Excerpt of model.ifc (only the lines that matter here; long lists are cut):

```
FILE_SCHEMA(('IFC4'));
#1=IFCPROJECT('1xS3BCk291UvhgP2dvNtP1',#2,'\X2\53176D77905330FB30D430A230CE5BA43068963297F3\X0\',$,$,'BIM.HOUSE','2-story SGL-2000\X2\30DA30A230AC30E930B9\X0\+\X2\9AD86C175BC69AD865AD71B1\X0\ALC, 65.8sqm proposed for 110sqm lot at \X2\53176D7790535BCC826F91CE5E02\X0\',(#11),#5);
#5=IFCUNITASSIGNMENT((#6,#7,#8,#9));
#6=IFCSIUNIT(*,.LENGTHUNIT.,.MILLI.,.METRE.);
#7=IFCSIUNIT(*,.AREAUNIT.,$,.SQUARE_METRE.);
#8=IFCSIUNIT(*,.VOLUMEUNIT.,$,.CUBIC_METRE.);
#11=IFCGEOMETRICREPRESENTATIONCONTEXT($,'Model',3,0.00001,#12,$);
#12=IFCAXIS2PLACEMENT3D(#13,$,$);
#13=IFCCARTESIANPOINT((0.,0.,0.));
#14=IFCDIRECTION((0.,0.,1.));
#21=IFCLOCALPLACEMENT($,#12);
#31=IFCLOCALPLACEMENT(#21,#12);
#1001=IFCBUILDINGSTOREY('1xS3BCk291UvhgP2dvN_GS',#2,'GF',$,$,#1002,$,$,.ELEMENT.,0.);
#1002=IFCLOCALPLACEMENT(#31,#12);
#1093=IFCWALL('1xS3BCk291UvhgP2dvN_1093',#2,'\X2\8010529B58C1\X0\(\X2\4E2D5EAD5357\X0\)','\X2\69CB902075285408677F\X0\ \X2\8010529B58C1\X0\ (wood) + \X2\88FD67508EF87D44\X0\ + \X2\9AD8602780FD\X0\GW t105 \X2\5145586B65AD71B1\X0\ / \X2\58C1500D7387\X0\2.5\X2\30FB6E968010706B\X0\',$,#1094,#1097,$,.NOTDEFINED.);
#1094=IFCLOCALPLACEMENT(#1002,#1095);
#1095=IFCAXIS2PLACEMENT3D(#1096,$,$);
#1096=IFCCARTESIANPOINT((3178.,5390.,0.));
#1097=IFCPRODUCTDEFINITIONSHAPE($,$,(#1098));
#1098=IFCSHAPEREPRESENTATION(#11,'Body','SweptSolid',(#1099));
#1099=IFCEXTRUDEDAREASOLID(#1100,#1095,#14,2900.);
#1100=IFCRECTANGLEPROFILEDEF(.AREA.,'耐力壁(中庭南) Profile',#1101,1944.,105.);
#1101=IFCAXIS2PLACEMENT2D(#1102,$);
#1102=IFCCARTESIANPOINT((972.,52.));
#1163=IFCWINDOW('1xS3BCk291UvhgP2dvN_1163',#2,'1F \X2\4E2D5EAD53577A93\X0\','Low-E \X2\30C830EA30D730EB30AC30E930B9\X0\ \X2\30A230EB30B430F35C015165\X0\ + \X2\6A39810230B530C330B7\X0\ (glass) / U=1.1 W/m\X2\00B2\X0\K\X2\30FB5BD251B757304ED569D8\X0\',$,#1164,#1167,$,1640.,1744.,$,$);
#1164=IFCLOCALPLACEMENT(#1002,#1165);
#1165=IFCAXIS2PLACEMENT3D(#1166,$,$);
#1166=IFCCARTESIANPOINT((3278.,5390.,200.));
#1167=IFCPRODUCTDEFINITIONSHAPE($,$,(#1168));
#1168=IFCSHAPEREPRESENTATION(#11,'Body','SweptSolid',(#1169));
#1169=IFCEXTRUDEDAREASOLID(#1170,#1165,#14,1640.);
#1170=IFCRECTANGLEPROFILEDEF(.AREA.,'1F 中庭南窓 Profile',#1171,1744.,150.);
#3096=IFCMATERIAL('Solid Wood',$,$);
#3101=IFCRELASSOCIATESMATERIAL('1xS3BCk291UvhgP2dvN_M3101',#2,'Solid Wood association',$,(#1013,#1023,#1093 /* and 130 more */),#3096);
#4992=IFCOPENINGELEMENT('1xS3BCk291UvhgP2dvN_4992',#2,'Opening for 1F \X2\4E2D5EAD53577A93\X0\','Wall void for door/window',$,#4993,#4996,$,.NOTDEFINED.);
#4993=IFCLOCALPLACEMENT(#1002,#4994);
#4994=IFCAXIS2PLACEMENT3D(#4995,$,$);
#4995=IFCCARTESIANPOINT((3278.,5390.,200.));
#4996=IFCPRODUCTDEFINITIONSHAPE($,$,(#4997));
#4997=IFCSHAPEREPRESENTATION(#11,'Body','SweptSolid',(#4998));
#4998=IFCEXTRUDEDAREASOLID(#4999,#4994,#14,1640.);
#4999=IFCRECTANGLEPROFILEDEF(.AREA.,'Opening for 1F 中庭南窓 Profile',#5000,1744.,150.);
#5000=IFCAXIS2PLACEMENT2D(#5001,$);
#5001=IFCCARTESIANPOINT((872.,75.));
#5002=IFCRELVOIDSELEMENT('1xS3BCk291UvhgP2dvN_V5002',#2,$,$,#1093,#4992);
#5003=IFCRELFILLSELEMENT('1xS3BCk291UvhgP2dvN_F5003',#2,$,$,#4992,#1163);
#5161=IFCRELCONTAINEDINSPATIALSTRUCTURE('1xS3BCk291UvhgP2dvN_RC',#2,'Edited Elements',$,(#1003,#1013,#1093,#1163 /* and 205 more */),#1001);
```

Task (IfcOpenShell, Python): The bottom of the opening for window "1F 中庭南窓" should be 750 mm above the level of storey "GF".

```python
import numpy as np
import ifcopenshell
import ifcopenshell.api.geometry
import ifcopenshell.geom
import ifcopenshell.util.element
import ifcopenshell.util.placement
import ifcopenshell.util.shape
import ifcopenshell.util.unit

model = ifcopenshell.open("model.ifc")
unit_scale = ifcopenshell.util.unit.calculate_unit_scale(model)

window = model.by_guid("1xS3BCk291UvhgP2dvN_1163")
opening = window.FillsVoids[0].RelatingOpeningElement
storey = ifcopenshell.util.element.get_container(window, ifc_class="IfcBuildingStorey")
level = ifcopenshell.util.placement.get_local_placement(storey.ObjectPlacement)[2, 3]

# The opening's origin need not be at the sill, so measure its lowest point.
shape = ifcopenshell.geom.create_shape(ifcopenshell.geom.settings(), opening)
bottom = ifcopenshell.util.shape.get_shape_bottom_elevation(shape, shape.geometry) / unit_scale
dz = level + 750.0 - bottom

shift = np.array([0.0, 0.0, dz])
# The window is not placed relative to its opening, so move both.
for product in (opening, window):
    matrix = ifcopenshell.util.placement.get_local_placement(product.ObjectPlacement)
    matrix[:3, 3] += shift
    ifcopenshell.api.geometry.edit_object_placement(model, product=product, matrix=matrix, is_si=False)

print(f"moved by {dz * unit_scale:+.3f} m")

model.write("model_edited.ifc")
```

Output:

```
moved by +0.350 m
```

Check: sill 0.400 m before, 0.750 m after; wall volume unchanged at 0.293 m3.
